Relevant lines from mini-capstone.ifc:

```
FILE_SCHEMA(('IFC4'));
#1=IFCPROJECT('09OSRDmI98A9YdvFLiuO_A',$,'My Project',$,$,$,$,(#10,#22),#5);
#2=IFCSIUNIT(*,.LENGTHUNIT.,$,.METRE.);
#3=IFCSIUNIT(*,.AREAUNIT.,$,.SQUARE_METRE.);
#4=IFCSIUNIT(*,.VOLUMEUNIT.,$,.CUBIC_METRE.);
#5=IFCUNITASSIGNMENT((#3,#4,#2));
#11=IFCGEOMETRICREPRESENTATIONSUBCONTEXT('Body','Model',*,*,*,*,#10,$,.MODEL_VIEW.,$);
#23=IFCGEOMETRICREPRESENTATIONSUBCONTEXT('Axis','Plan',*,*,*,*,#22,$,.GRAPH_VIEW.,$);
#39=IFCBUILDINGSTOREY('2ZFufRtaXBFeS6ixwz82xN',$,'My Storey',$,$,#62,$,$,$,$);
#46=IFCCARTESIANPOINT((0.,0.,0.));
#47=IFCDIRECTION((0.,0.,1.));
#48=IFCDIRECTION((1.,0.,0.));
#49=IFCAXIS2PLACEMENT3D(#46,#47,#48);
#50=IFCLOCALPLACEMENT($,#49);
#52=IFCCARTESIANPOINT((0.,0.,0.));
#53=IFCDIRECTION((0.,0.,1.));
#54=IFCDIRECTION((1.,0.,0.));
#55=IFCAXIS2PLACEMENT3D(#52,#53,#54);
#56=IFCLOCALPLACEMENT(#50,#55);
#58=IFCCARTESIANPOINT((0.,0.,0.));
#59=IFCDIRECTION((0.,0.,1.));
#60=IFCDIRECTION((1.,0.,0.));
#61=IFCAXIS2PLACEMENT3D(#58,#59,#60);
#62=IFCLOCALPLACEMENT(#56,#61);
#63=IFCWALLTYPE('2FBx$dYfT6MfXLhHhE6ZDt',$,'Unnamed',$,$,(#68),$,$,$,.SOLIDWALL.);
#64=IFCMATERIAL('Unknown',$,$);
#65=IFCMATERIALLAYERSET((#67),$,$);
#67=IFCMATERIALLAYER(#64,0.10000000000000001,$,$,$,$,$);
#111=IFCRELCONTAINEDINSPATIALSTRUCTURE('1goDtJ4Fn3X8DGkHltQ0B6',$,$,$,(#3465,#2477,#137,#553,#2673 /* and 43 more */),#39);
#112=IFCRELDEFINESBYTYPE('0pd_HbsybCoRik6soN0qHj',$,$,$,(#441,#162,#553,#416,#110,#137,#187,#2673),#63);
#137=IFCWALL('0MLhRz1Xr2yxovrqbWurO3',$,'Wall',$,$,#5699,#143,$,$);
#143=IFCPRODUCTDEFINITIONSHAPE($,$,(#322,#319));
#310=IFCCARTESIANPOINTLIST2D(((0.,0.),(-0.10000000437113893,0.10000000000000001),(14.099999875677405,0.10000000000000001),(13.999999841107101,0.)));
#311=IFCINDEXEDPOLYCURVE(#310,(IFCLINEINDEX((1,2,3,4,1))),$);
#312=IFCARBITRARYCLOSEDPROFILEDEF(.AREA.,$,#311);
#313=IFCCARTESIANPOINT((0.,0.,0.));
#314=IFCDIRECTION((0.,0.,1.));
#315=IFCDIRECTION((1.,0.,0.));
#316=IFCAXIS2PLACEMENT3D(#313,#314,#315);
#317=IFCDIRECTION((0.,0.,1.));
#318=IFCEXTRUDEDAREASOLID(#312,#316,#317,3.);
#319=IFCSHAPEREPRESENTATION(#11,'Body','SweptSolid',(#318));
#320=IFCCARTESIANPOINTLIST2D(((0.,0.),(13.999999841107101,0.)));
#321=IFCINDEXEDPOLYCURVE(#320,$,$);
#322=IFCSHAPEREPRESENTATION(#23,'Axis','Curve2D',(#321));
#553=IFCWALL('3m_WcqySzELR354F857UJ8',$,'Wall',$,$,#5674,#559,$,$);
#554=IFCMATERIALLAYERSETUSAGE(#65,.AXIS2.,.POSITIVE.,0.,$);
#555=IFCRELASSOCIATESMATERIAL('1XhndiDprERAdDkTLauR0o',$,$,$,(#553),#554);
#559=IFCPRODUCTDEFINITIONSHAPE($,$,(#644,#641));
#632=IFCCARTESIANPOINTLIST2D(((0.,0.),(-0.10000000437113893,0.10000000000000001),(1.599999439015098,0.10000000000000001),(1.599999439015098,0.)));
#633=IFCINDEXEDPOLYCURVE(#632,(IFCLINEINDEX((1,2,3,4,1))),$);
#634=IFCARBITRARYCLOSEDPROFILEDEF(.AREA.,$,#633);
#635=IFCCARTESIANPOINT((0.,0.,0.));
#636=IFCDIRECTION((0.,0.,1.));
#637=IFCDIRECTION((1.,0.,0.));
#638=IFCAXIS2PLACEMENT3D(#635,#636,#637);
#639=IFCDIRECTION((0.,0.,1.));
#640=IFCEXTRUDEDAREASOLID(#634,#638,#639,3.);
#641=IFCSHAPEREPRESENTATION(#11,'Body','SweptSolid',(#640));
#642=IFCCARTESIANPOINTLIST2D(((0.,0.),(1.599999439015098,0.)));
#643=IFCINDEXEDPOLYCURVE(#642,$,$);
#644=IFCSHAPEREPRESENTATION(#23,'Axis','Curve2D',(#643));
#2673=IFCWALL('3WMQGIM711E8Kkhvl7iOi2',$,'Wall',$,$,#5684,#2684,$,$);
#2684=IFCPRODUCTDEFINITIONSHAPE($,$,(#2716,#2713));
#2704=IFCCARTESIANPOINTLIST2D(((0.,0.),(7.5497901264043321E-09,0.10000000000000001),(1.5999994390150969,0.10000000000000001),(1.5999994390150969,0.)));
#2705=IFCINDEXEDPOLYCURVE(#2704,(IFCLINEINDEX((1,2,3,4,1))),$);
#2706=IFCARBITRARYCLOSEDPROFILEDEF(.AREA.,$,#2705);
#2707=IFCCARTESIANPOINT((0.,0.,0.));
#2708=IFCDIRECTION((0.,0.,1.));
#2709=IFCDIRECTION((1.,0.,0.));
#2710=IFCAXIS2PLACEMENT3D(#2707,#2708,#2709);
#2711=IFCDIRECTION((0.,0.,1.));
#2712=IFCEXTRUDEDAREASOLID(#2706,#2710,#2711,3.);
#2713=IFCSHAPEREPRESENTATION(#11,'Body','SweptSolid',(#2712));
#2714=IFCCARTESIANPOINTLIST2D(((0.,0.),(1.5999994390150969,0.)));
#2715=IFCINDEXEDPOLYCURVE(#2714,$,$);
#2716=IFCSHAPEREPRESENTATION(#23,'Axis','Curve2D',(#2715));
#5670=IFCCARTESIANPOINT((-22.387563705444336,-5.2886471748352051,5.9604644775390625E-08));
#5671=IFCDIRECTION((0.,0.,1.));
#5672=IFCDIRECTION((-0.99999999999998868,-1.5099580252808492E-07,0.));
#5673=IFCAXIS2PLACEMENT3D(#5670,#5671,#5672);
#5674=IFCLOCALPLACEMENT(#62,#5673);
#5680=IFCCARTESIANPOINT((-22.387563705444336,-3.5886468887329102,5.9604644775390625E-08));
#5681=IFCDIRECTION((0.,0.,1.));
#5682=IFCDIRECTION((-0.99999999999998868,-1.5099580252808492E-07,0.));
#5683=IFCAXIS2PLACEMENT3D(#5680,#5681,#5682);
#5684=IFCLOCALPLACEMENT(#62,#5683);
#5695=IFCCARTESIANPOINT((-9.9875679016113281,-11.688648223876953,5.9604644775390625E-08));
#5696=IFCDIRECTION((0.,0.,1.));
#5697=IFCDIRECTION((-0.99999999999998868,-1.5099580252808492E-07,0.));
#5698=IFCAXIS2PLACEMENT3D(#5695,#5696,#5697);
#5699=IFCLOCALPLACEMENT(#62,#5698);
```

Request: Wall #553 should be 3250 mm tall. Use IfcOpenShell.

```python
import ifcopenshell
import ifcopenshell.geom
import ifcopenshell.util.representation
import ifcopenshell.util.shape
import ifcopenshell.util.unit

model = ifcopenshell.open("mini-capstone.ifc")
unit_scale = ifcopenshell.util.unit.calculate_unit_scale(model)
settings = ifcopenshell.geom.settings()


def volume(element):
    """Net volume in cubic metres, openings subtracted."""
    shape = ifcopenshell.geom.create_shape(settings, element)
    return ifcopenshell.util.shape.get_volume(shape.geometry)


wall = model.by_guid("3m_WcqySzELR354F857UJ8")
before = volume(wall)

body = ifcopenshell.util.representation.get_representation(wall, "Model", "Body")
solid = body.Items[0]
old_height = solid.Depth
solid.Depth = 3.25 / unit_scale
after = volume(wall)

print(f"height {old_height:g} -> {solid.Depth:g}, volume {before:.3f} -> {after:.3f} m3")

model.write("mini-capstone_edited.ifc")
```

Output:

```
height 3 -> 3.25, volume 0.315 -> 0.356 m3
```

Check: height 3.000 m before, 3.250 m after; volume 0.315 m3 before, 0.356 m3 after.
